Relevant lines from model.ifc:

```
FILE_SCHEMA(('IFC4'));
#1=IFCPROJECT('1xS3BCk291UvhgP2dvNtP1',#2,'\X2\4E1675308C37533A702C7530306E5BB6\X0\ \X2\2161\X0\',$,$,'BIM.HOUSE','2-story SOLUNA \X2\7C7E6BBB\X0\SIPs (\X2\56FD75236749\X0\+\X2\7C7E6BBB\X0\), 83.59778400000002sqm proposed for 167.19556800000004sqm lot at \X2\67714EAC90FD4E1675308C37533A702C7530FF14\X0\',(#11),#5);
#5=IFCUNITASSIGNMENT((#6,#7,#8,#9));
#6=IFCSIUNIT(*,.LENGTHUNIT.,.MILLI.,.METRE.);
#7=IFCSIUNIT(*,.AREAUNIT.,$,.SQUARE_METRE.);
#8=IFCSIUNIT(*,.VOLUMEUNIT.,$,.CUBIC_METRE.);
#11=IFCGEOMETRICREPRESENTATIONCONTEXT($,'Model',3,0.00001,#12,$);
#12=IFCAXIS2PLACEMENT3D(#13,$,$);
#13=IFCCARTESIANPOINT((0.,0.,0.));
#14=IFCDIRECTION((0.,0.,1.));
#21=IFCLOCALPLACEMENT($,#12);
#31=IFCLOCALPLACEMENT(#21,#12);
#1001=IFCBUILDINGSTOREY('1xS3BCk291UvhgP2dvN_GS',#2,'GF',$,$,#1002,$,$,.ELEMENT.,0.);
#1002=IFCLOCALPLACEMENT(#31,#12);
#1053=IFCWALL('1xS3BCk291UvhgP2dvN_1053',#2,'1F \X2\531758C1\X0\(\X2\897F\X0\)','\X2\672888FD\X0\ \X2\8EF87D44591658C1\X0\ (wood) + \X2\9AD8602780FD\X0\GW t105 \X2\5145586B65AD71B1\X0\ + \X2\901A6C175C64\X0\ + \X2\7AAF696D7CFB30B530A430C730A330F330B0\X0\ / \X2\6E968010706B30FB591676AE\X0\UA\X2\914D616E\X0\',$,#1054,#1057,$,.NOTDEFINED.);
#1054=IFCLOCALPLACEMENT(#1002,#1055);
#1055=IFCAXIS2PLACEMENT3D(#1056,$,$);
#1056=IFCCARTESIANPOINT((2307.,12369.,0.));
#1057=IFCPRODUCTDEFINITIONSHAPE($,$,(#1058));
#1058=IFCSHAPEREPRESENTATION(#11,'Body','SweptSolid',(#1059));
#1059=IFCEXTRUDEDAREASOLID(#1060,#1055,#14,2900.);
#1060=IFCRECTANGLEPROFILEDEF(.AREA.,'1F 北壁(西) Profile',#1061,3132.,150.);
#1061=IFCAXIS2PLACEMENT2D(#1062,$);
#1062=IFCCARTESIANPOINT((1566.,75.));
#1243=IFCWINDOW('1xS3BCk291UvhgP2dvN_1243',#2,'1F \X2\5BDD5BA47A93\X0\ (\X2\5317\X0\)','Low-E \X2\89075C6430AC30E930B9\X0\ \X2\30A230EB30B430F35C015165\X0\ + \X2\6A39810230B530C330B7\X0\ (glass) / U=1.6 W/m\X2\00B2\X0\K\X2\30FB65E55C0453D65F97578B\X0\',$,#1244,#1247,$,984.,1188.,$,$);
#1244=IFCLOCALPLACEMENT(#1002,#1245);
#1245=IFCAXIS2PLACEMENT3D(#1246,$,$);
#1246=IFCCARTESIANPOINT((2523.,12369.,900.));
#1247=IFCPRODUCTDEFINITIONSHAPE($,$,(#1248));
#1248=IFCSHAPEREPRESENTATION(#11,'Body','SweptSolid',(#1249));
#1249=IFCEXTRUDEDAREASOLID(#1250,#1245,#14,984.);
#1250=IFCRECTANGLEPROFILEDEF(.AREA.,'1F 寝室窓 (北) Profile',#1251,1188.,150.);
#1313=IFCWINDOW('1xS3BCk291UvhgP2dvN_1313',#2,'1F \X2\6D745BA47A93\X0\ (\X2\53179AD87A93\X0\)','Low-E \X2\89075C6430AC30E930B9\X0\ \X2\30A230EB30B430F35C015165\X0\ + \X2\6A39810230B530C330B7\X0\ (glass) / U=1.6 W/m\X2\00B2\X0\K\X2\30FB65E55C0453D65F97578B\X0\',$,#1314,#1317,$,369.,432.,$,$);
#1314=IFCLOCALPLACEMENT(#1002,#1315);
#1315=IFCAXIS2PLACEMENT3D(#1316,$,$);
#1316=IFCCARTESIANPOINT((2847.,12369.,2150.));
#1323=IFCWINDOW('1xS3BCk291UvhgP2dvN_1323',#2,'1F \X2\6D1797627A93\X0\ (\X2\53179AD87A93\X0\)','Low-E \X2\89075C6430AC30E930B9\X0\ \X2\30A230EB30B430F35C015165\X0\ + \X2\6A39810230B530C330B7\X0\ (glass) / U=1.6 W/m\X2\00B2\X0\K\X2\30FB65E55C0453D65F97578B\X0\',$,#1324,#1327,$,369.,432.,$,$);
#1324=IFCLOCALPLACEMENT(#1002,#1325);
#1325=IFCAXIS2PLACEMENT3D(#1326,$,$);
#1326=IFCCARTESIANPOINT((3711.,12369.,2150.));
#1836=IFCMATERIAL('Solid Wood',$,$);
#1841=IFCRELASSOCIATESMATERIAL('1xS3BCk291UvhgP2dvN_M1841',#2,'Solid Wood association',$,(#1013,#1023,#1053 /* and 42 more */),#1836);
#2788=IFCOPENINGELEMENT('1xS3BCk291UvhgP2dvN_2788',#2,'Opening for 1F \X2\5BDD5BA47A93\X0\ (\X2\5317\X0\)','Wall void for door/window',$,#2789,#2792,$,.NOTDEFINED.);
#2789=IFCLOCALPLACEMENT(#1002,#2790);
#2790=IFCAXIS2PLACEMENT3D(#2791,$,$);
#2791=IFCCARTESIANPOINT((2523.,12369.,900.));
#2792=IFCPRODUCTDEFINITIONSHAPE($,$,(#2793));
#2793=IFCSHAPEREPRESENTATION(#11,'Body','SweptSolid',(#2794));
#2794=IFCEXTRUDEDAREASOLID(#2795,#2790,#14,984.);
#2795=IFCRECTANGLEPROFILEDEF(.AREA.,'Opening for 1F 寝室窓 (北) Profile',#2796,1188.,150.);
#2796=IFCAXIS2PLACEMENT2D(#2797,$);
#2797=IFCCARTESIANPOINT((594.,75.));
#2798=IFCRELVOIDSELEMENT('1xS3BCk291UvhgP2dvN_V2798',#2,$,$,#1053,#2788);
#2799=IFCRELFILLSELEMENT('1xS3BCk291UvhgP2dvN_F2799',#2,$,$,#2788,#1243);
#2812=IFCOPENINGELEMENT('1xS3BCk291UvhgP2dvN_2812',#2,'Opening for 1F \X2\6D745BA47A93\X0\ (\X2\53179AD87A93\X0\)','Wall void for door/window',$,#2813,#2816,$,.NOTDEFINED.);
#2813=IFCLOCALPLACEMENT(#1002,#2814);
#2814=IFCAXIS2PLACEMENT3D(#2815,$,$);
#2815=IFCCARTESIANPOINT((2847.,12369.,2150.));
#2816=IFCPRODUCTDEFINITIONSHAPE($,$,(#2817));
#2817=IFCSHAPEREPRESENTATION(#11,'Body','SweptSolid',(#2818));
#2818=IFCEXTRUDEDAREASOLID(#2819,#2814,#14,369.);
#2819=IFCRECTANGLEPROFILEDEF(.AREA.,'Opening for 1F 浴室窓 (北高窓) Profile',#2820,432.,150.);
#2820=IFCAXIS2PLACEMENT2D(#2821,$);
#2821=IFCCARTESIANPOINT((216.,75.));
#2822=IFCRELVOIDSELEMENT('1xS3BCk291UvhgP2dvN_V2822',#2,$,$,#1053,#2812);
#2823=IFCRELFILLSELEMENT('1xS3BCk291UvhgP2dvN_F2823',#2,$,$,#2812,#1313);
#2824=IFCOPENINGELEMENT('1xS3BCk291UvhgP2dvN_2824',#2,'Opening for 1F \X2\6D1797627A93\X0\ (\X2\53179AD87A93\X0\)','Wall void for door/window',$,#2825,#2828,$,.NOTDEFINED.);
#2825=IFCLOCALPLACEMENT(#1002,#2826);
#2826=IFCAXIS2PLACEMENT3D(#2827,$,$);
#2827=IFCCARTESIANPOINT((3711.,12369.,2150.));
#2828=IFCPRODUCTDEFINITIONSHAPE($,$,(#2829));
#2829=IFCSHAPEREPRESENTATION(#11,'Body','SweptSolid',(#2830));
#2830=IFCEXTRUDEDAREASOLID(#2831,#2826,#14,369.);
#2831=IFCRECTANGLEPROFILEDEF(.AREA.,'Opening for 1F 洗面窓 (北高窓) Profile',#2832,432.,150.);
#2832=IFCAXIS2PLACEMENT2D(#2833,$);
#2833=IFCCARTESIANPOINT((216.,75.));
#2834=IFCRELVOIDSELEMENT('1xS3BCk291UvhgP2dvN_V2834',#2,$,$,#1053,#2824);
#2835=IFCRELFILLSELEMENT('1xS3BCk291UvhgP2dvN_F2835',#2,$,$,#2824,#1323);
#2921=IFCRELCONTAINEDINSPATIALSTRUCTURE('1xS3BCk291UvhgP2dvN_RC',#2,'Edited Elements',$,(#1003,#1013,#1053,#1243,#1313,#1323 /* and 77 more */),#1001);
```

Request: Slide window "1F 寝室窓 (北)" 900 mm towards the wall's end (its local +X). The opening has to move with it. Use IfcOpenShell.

```python
import ifcopenshell
import ifcopenshell.api.geometry
import ifcopenshell.util.placement
import ifcopenshell.util.unit

model = ifcopenshell.open("model.ifc")
unit_scale = ifcopenshell.util.unit.calculate_unit_scale(model)

window = model.by_guid("1xS3BCk291UvhgP2dvN_1243")
opening = window.FillsVoids[0].RelatingOpeningElement
wall = opening.VoidsElements[0].RelatingBuildingElement

wall_matrix = ifcopenshell.util.placement.get_local_placement(wall.ObjectPlacement)
shift = wall_matrix[:3, 0] * 0.9 / unit_scale
before = ifcopenshell.util.placement.get_local_placement(window.ObjectPlacement)[:3, 3].copy()

# The window is not placed relative to its opening, so move both.
for product in (opening, window):
    matrix = ifcopenshell.util.placement.get_local_placement(product.ObjectPlacement)
    matrix[:3, 3] += shift
    ifcopenshell.api.geometry.edit_object_placement(model, product=product, matrix=matrix, is_si=False)

after = ifcopenshell.util.placement.get_local_placement(window.ObjectPlacement)[:3, 3]
print("window moved by", (after - before).round(3) + 0.0)

model.write("model_updated.ifc")
```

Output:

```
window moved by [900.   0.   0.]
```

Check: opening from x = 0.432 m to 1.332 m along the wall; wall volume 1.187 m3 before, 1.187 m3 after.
